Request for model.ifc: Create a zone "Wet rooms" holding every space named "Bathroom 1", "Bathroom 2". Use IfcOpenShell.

First a look at what the model holds.

```python
import ifcopenshell

model = ifcopenshell.open("model.ifc")
print(model.schema)
seen = {}
for space in model.by_type("IfcSpace"):
    seen[space.LongName] = seen.get(space.LongName, 0) + 1
for name, count in sorted(seen.items(), key=str):
    print(count, "x", name)
print("zones:", [z.Name for z in model.by_type("IfcZone")][:20])
```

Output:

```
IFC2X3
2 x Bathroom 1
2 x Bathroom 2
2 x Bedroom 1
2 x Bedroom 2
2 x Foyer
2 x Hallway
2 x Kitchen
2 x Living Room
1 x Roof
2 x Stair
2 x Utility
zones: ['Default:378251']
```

```python
import ifcopenshell
import ifcopenshell.api.group
import ifcopenshell.api.root

model = ifcopenshell.open("model.ifc")

names = {"Bathroom 1", "Bathroom 2"}
spaces = [s for s in model.by_type("IfcSpace") if s.LongName in names]

zone = ifcopenshell.api.root.create_entity(model, ifc_class="IfcZone", name="Wet rooms")
ifcopenshell.api.group.assign_group(model, products=spaces, group=zone)
print(len(spaces), "spaces in", zone.Name)

model.write("model_rev.ifc")
```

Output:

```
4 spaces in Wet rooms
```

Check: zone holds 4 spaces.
